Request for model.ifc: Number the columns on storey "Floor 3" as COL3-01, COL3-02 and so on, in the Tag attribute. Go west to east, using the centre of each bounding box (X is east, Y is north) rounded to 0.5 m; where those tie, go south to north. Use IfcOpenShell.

First a look at what the model holds.

```python
import ifcopenshell
import ifcopenshell.util.element
import ifcopenshell.util.placement

model = ifcopenshell.open("model.ifc")
print(model.schema)
storey = next(s for s in model.by_type("IfcBuildingStorey") if s.Name == "Floor 3")
columns = [e for e in ifcopenshell.util.element.get_decomposition(storey) if e.is_a("IfcColumn")]
for e in sorted(columns, key=lambda e: e.id()):
    origin = ifcopenshell.util.placement.get_local_placement(e.ObjectPlacement)[:3, 3]
    print(e.id(), e.Tag, e.Name, origin.round(2) + 0.0, sep=" | ")
```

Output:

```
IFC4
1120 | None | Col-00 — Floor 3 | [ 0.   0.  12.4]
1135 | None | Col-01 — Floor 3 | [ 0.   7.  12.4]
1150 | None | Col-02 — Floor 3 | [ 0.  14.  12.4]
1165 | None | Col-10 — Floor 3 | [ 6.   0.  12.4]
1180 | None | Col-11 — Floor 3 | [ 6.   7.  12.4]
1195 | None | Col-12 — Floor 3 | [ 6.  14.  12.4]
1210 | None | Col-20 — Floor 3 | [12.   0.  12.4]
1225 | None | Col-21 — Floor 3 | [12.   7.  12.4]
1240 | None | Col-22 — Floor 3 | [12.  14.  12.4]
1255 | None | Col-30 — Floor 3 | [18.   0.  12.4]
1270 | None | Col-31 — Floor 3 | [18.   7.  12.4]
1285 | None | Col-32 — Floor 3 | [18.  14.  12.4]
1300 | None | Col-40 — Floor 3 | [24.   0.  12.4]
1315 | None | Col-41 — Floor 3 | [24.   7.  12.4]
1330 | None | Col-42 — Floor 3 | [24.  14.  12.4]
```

```python
import ifcopenshell
import ifcopenshell.geom
import ifcopenshell.util.element
import ifcopenshell.util.shape

model = ifcopenshell.open("model.ifc")
settings = ifcopenshell.geom.settings()
settings.set("use-world-coords", True)


def centre(element):
    shape = ifcopenshell.geom.create_shape(settings, element)
    return ifcopenshell.util.shape.get_bbox_centroid(shape.geometry)


storey = next(s for s in model.by_type("IfcBuildingStorey") if s.Name == "Floor 3")
columns = [e for e in ifcopenshell.util.element.get_decomposition(storey) if e.is_a("IfcColumn")]

# Insertion points can sit at a corner or the storey origin, so sort by the geometry (in metres).
centres = {e: centre(e) for e in columns}
columns.sort(key=lambda e: (round(centres[e][0] / 0.5), centres[e][1]))

for i, e in enumerate(columns, start=1):
    number = f"COL3-{i:02d}"
    e.Tag = number
    print(e.id(), number)

model.write("model_v2.ifc")
```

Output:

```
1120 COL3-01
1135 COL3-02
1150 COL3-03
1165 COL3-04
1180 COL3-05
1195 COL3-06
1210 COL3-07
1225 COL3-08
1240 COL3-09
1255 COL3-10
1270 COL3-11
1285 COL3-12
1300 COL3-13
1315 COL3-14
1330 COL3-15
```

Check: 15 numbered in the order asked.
